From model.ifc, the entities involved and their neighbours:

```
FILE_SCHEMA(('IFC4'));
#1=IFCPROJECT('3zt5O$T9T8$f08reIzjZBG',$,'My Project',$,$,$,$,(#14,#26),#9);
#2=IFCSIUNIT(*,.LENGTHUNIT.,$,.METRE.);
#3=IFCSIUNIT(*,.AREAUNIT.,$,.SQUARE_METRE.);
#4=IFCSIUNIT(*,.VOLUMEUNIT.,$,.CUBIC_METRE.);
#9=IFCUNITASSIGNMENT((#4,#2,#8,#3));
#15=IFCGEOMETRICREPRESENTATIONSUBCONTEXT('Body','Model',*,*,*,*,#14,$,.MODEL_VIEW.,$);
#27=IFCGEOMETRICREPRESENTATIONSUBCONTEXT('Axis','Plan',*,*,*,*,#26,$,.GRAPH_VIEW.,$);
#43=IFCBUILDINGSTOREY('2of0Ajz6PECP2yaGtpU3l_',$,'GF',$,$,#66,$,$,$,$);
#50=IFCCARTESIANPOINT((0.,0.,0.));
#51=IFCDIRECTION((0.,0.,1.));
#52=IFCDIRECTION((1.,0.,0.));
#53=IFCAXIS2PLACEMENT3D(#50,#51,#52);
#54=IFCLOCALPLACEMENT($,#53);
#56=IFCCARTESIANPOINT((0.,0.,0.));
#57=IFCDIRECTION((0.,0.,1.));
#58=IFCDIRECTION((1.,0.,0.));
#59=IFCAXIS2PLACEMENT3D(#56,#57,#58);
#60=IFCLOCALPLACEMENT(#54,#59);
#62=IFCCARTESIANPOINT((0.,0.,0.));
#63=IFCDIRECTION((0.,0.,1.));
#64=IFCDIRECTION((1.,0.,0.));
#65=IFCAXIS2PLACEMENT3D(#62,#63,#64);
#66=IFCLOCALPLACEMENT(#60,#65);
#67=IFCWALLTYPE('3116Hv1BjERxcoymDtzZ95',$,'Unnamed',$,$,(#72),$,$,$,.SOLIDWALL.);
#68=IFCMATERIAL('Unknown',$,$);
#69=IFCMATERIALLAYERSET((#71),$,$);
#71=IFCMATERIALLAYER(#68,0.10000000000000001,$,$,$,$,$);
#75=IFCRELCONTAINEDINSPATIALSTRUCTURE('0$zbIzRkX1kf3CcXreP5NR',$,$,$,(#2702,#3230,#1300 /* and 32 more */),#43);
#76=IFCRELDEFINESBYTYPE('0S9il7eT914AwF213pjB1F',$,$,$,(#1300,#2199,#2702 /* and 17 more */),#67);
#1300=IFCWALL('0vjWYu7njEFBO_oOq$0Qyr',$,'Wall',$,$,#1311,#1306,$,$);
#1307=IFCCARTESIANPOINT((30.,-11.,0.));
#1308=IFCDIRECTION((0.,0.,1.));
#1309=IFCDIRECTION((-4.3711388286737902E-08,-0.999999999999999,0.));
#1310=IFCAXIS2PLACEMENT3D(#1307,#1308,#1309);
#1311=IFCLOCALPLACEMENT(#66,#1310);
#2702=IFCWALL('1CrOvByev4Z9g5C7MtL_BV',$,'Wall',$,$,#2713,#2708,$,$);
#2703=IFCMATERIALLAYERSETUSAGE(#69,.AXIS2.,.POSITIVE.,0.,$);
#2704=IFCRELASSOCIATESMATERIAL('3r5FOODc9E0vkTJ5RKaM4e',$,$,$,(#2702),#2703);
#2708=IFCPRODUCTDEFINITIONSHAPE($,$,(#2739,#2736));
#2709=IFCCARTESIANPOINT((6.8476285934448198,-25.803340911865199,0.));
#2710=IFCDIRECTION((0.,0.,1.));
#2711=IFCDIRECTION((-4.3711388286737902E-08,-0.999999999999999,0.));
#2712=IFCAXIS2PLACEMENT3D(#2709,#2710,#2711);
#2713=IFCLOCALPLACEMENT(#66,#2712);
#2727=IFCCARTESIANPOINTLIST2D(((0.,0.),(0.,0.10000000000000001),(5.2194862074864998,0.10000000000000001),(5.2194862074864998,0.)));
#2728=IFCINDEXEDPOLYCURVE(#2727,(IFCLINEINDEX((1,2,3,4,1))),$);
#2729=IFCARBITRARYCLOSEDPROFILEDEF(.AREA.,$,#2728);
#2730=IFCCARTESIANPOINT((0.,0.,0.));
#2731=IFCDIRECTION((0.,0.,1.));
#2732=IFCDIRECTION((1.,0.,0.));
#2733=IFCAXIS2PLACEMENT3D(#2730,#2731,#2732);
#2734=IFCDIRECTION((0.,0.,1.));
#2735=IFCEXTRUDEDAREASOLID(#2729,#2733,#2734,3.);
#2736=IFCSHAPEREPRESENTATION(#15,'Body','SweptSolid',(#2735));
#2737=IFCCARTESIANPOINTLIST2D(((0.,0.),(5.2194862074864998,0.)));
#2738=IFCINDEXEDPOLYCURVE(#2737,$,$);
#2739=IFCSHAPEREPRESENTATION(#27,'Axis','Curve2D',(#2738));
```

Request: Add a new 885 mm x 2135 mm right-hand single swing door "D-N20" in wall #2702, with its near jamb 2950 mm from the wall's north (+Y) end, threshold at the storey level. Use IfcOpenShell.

```python
import numpy as np
import ifcopenshell
import ifcopenshell.api.feature
import ifcopenshell.api.geometry
import ifcopenshell.api.root
import ifcopenshell.api.spatial
import ifcopenshell.geom
import ifcopenshell.util.element
import ifcopenshell.util.placement
import ifcopenshell.util.representation
import ifcopenshell.util.shape
import ifcopenshell.util.unit

model = ifcopenshell.open("model.ifc")
unit_scale = ifcopenshell.util.unit.calculate_unit_scale(model)
settings = ifcopenshell.geom.settings()


def volume(element):
    """Net volume in cubic metres, openings subtracted."""
    shape = ifcopenshell.geom.create_shape(settings, element)
    return ifcopenshell.util.shape.get_volume(shape.geometry)


wall = model.by_id(2702)
storey = ifcopenshell.util.element.get_container(wall, ifc_class="IfcBuildingStorey")
context = ifcopenshell.util.representation.get_context(model, "Model", "Body", "MODEL_VIEW")
before = volume(wall)

width, height, from_end, sill = 0.885, 2.135, 2.95, 0.0  # metres

# The wall runs along its own X axis, and the end named is its -X end.
wall_shape = ifcopenshell.geom.create_shape(settings, wall)
x, y, z = ifcopenshell.util.shape.get_vertices(wall_shape.geometry).T
start = x.min() + from_end
face, thickness = float(y.min()), float(y.max() - y.min())
wall_matrix = ifcopenshell.util.placement.get_local_placement(wall.ObjectPlacement)
level = ifcopenshell.util.placement.get_local_placement(storey.ObjectPlacement)[2, 3]


def in_wall(x, y):
    """Placement at x, y metres in the wall's axes, at sill height."""
    matrix = wall_matrix.copy()
    matrix[:, 3] = wall_matrix @ np.array([x / unit_scale, y / unit_scale, 0.0, 1.0])
    matrix[2, 3] = level + sill / unit_scale
    return matrix


# Opening: a box that overshoots both wall faces by 50 mm.
opening = ifcopenshell.api.root.create_entity(model, ifc_class="IfcOpeningElement", predefined_type="OPENING")
box = ifcopenshell.api.geometry.add_wall_representation(
    model, context=context, length=width, height=height, thickness=thickness + 0.1
)
ifcopenshell.api.geometry.assign_representation(model, product=opening, representation=box)
ifcopenshell.api.geometry.edit_object_placement(model, product=opening, matrix=in_wall(start, face - 0.05), is_si=False)
ifcopenshell.api.feature.add_feature(model, feature=opening, element=wall)

door = ifcopenshell.api.root.create_entity(model, ifc_class="IfcDoor", name="D-N20", predefined_type="DOOR")
door.OverallWidth, door.OverallHeight = width / unit_scale, height / unit_scale
door.OperationType = "SINGLE_SWING_RIGHT"
body = ifcopenshell.api.geometry.add_door_representation(
    model,
    context=context,
    overall_width=door.OverallWidth,
    overall_height=door.OverallHeight,
    operation_type="SINGLE_SWING_RIGHT",
    lining_properties={"LiningDepth": thickness / unit_scale, "ThresholdDepth": thickness / unit_scale},
)
ifcopenshell.api.geometry.assign_representation(model, product=door, representation=body)
ifcopenshell.api.spatial.assign_container(model, products=[door], relating_structure=storey)
ifcopenshell.api.feature.add_filling(model, opening=opening, element=door)

# The lining spans the wall, so the door starts at the wall face.
ifcopenshell.api.geometry.edit_object_placement(model, product=door, matrix=in_wall(start, face), is_si=False)

after = volume(wall)

print(f"wall volume {before:.3f} -> {after:.3f} m3")

model.write("model_rev.ifc")
```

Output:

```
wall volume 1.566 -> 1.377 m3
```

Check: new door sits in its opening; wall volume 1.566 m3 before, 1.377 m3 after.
